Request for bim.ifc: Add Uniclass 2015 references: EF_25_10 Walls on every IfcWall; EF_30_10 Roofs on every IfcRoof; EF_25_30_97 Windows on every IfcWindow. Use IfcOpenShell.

First a look at what the model holds.

```python
import ifcopenshell

model = ifcopenshell.open("bim.ifc")
print(model.schema)
print("classifications:", [c.Name for c in model.by_type("IfcClassification")])
for ifc_class in ("IfcDoor", "IfcRoof", "IfcStair", "IfcWall", "IfcWindow"):
    print(ifc_class, len(model.by_type(ifc_class)))
```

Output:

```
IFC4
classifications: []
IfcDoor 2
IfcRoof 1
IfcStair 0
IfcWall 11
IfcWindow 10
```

```python
import ifcopenshell
import ifcopenshell.api.classification

model = ifcopenshell.open("bim.ifc")

system = ifcopenshell.api.classification.add_classification(model, classification="Uniclass 2015")

codes = {
    "IfcWall": ("EF_25_10", "Walls"),
    "IfcRoof": ("EF_30_10", "Roofs"),
    "IfcWindow": ("EF_25_30_97", "Windows"),
}
for ifc_class, (code, name) in codes.items():
    products = model.by_type(ifc_class)
    ifcopenshell.api.classification.add_reference(
        model, products=products, classification=system, identification=code, name=name
    )
    print(code, len(products))

model.write("bim_edited.ifc")
```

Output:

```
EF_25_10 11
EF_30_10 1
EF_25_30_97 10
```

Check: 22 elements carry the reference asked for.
